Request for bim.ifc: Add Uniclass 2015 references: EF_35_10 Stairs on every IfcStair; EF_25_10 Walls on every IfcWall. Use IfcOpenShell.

First a look at what the model holds.

```python
import ifcopenshell

model = ifcopenshell.open("bim.ifc")
print(model.schema)
print("classifications:", [c.Name for c in model.by_type("IfcClassification")])
for ifc_class in ("IfcDoor", "IfcRoof", "IfcStair", "IfcWall", "IfcWindow"):
    print(ifc_class, len(model.by_type(ifc_class)))
```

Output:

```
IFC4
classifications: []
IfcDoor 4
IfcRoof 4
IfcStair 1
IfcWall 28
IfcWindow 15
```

```python
import ifcopenshell
import ifcopenshell.api.classification

model = ifcopenshell.open("bim.ifc")

system = ifcopenshell.api.classification.add_classification(model, classification="Uniclass 2015")

codes = {
    "IfcStair": ("EF_35_10", "Stairs"),
    "IfcWall": ("EF_25_10", "Walls"),
}
for ifc_class, (code, name) in codes.items():
    products = model.by_type(ifc_class)
    ifcopenshell.api.classification.add_reference(
        model, products=products, classification=system, identification=code, name=name
    )
    print(code, len(products))

model.write("bim_updated.ifc")
```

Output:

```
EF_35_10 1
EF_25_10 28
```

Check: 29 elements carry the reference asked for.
